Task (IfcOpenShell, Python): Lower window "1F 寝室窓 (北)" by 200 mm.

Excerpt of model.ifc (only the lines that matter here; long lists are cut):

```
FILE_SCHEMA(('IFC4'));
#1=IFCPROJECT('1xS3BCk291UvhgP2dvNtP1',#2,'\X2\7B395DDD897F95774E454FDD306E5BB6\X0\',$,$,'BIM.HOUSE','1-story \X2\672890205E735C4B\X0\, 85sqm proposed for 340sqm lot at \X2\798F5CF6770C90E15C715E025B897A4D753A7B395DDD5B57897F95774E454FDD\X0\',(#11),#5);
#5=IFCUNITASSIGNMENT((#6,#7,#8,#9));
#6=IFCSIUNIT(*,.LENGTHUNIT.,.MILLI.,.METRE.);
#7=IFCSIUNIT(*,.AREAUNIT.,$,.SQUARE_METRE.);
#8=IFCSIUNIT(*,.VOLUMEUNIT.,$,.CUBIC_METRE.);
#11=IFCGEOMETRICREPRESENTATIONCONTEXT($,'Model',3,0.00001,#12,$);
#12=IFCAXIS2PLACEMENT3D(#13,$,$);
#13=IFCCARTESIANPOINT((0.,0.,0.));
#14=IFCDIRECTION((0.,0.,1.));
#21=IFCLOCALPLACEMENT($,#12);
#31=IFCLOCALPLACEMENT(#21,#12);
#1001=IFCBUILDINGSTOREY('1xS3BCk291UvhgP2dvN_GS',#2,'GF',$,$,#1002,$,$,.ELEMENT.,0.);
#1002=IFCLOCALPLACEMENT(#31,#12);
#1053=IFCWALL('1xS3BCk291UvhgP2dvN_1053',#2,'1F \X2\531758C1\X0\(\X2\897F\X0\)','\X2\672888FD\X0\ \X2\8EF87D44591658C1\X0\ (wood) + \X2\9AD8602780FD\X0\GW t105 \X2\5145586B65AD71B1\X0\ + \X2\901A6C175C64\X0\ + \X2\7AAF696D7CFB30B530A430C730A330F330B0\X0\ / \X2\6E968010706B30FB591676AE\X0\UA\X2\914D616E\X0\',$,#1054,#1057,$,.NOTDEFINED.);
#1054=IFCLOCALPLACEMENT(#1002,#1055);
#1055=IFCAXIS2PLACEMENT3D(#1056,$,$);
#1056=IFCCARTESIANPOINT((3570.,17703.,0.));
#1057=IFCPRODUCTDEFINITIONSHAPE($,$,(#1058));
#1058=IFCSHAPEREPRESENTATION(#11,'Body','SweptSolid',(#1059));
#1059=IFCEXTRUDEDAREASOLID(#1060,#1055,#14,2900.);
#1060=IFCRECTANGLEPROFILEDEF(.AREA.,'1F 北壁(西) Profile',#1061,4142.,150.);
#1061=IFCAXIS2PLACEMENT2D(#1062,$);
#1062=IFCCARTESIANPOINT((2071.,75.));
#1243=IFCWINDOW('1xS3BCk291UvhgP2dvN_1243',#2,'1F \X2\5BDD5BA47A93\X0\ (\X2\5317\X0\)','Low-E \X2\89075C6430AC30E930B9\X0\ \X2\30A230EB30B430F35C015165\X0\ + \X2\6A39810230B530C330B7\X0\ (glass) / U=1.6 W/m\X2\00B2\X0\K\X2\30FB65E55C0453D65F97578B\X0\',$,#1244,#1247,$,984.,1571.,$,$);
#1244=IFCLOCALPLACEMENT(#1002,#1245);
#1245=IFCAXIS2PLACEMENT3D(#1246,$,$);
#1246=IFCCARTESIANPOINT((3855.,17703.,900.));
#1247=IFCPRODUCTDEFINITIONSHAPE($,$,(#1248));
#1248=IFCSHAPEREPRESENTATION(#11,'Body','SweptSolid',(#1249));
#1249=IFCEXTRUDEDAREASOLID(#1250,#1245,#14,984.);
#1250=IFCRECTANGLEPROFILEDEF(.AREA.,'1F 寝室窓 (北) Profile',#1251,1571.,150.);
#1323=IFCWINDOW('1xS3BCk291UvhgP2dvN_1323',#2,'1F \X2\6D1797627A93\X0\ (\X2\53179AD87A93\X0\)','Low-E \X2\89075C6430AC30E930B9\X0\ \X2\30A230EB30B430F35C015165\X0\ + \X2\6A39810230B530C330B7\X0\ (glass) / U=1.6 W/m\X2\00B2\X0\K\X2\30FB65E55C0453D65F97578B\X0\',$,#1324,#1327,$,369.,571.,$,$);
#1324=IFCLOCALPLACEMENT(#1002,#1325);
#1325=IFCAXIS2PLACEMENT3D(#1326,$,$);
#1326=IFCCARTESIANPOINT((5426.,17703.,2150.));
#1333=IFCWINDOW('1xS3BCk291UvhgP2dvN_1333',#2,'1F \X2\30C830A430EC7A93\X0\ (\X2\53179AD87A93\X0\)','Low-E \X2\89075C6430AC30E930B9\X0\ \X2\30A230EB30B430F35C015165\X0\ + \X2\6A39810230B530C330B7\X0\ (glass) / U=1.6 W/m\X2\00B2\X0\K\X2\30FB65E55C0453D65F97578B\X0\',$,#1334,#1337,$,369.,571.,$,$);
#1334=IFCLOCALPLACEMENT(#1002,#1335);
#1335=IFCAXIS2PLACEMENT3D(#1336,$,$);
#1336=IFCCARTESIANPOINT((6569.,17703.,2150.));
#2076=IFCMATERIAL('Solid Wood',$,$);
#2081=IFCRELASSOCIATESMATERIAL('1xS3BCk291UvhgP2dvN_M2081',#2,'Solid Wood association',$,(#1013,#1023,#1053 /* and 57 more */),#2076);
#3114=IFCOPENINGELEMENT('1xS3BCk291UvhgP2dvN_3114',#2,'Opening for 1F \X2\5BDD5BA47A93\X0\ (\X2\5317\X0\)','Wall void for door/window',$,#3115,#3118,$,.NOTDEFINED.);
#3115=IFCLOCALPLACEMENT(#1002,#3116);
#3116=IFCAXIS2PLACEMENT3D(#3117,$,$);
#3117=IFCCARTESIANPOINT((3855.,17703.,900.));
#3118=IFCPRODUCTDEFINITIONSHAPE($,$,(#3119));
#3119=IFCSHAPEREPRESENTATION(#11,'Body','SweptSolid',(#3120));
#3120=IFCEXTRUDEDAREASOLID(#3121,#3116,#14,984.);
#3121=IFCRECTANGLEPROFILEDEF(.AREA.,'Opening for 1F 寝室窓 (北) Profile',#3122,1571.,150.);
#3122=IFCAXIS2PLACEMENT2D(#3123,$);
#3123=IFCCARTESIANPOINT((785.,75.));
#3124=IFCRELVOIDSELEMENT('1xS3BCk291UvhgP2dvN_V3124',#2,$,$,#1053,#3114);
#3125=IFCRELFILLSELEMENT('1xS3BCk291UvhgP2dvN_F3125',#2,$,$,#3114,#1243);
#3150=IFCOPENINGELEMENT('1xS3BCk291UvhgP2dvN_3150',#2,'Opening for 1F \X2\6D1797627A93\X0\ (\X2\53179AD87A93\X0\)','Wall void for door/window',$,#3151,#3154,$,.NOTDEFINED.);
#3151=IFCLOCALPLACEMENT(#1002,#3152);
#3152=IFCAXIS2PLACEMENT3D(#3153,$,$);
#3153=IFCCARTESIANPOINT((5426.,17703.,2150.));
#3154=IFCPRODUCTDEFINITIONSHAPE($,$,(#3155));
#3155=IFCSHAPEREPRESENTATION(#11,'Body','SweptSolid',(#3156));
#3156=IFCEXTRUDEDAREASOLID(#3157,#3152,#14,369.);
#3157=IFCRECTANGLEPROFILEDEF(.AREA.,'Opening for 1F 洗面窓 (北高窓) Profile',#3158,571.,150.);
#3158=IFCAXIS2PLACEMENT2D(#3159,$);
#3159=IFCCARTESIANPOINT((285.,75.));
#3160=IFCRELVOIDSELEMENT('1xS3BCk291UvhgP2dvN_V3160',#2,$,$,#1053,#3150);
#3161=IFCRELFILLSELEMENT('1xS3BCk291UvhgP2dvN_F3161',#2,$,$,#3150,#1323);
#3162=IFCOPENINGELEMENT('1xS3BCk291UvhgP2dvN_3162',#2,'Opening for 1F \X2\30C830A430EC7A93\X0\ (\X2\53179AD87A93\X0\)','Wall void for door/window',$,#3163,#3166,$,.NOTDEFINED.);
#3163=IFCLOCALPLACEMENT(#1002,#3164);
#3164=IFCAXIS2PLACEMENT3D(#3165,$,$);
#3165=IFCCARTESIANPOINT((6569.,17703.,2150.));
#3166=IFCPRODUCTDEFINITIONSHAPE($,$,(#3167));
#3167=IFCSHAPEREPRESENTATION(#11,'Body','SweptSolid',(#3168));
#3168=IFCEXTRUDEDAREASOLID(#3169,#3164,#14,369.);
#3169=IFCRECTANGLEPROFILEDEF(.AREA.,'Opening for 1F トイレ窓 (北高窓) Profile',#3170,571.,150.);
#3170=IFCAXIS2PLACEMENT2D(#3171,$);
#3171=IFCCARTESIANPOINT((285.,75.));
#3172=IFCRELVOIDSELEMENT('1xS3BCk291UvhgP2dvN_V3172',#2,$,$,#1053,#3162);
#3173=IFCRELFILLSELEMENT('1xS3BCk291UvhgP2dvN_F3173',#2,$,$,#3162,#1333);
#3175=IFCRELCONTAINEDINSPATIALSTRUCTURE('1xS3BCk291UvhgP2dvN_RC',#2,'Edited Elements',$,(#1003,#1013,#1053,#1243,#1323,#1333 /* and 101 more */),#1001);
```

```python
import numpy as np
import ifcopenshell
import ifcopenshell.api.geometry
import ifcopenshell.util.placement
import ifcopenshell.util.unit

model = ifcopenshell.open("model.ifc")
unit_scale = ifcopenshell.util.unit.calculate_unit_scale(model)

window = model.by_guid("1xS3BCk291UvhgP2dvN_1243")
opening = window.FillsVoids[0].RelatingOpeningElement
dz = -0.2 / unit_scale

shift = np.array([0.0, 0.0, dz])
# The window is not placed relative to its opening, so move both.
for product in (opening, window):
    matrix = ifcopenshell.util.placement.get_local_placement(product.ObjectPlacement)
    matrix[:3, 3] += shift
    ifcopenshell.api.geometry.edit_object_placement(model, product=product, matrix=matrix, is_si=False)

print(f"moved by {dz * unit_scale:+.3f} m")

model.write("model-out.ifc")
```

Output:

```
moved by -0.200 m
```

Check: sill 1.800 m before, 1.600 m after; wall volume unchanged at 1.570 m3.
